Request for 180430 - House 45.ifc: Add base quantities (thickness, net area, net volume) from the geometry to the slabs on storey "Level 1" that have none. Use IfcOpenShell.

First a look at what the model holds.

```python
import ifcopenshell
import ifcopenshell.util.element
import ifcopenshell.util.unit

model = ifcopenshell.open("180430 - House 45.ifc")
print(model.schema)
for unit_type in ("LENGTHUNIT", "AREAUNIT", "VOLUMEUNIT"):
    print(unit_type, ifcopenshell.util.unit.calculate_unit_scale(model, unit_type))
storey = next(s for s in model.by_type("IfcBuildingStorey") if s.Name == "Level 1")
slabs = [e for e in ifcopenshell.util.element.get_decomposition(storey) if e.is_a("IfcSlab")]
for e in sorted(slabs, key=lambda e: e.id()):
    print(e.id(), e.is_a(), e.Name, list(ifcopenshell.util.element.get_psets(e, qtos_only=True)), sep=" | ")
```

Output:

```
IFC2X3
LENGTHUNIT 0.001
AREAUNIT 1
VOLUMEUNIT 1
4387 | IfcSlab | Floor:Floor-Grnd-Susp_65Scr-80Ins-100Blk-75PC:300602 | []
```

```python
import ifcopenshell
import ifcopenshell.api.pset
import ifcopenshell.geom
import ifcopenshell.util.element
import ifcopenshell.util.shape
import ifcopenshell.util.unit

model = ifcopenshell.open("180430 - House 45.ifc")
unit_scale = ifcopenshell.util.unit.calculate_unit_scale(model)
area_scale = ifcopenshell.util.unit.calculate_unit_scale(model, "AREAUNIT")
volume_scale = ifcopenshell.util.unit.calculate_unit_scale(model, "VOLUMEUNIT")
settings = ifcopenshell.geom.settings()

storey = next(s for s in model.by_type("IfcBuildingStorey") if s.Name == "Level 1")
slabs = [e for e in ifcopenshell.util.element.get_decomposition(storey) if e.is_a("IfcSlab")]

for e in sorted(slabs, key=lambda e: e.id()):
    if ifcopenshell.util.element.get_psets(e, qtos_only=True, should_inherit=False):
        continue
    # Geometry comes back in metres, in the element's own axes.
    shape = ifcopenshell.geom.create_shape(settings, e)
    values = {
        "Width": ifcopenshell.util.shape.get_z(shape.geometry) / unit_scale,
        "NetArea": ifcopenshell.util.shape.get_footprint_area(shape.geometry) / area_scale,
        "NetVolume": ifcopenshell.util.shape.get_volume(shape.geometry) / volume_scale,
    }
    qto = ifcopenshell.api.pset.add_qto(model, product=e, name="BaseQuantities")
    ifcopenshell.api.pset.edit_qto(model, qto=qto, properties=values)
    print(e.id(), {k: round(v, 3) for k, v in values.items()})

model.write("180430 - House 45_updated.ifc")
```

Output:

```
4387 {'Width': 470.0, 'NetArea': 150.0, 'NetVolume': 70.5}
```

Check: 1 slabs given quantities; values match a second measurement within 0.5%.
